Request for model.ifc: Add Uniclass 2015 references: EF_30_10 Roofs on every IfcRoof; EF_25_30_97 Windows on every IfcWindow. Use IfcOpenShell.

First a look at what the model holds.

```python
import ifcopenshell

model = ifcopenshell.open("model.ifc")
print(model.schema)
print("classifications:", [c.Name for c in model.by_type("IfcClassification")])
for ifc_class in ("IfcDoor", "IfcRoof", "IfcStair", "IfcWall", "IfcWindow"):
    print(ifc_class, len(model.by_type(ifc_class)))
```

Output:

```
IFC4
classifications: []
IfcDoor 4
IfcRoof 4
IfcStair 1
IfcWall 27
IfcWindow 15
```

```python
import ifcopenshell
import ifcopenshell.api.classification

model = ifcopenshell.open("model.ifc")

system = ifcopenshell.api.classification.add_classification(model, classification="Uniclass 2015")

codes = {
    "IfcRoof": ("EF_30_10", "Roofs"),
    "IfcWindow": ("EF_25_30_97", "Windows"),
}
for ifc_class, (code, name) in codes.items():
    products = model.by_type(ifc_class)
    ifcopenshell.api.classification.add_reference(
        model, products=products, classification=system, identification=code, name=name
    )
    print(code, len(products))

model.write("model_edited.ifc")
```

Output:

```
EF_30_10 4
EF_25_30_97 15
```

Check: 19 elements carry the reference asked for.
